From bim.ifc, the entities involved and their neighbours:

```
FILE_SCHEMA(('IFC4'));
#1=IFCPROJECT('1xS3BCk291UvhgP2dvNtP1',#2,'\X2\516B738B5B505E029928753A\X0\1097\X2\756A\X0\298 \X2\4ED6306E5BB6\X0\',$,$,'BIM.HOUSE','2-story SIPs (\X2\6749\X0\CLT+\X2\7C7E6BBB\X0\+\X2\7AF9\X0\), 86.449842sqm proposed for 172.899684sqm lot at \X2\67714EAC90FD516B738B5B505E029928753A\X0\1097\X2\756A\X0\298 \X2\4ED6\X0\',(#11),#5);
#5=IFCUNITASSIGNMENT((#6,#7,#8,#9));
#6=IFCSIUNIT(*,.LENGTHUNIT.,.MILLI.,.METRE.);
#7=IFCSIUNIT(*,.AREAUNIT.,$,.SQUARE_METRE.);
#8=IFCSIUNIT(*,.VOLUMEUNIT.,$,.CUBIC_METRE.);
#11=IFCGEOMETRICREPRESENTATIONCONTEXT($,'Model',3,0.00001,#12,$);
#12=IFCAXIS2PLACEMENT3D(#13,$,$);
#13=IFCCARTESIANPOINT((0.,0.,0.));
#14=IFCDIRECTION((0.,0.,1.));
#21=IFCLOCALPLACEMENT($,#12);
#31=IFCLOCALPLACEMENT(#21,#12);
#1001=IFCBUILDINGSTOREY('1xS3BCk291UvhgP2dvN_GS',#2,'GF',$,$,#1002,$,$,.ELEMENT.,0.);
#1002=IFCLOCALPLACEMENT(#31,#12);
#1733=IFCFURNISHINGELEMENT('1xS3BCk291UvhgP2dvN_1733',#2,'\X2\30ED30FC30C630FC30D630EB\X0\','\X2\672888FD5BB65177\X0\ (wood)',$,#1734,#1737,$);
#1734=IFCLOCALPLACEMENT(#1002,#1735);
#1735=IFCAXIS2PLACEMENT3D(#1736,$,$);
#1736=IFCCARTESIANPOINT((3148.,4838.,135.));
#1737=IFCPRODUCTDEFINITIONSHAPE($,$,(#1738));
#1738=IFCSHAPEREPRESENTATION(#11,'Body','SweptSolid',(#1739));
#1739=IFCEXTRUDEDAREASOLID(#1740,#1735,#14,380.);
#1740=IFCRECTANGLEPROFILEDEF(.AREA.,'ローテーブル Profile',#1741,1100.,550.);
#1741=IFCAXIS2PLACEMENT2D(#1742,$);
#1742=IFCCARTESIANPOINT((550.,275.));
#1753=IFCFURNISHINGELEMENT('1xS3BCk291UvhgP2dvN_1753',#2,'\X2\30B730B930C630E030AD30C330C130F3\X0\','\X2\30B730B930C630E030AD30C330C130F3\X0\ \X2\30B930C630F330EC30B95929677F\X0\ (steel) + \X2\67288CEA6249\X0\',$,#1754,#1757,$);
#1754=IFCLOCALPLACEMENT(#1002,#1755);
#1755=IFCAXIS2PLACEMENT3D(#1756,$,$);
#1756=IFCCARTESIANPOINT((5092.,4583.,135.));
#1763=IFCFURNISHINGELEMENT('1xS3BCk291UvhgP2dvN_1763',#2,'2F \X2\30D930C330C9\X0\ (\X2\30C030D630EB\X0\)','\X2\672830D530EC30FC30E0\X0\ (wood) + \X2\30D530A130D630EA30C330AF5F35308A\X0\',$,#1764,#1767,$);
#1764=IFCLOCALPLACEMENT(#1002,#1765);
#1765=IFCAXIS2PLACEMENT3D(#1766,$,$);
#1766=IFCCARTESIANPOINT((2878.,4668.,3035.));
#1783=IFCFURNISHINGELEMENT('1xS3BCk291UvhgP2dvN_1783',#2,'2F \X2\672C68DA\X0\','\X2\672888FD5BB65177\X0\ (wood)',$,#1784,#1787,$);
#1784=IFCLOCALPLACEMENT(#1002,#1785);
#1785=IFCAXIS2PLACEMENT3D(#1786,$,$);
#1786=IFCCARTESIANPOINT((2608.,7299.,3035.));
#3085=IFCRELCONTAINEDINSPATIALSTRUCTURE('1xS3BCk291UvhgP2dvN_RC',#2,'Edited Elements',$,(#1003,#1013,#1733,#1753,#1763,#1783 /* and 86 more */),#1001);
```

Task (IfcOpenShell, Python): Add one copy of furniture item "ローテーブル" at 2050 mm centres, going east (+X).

```python
import numpy as np
import ifcopenshell
import ifcopenshell.api.geometry
import ifcopenshell.api.root
import ifcopenshell.util.element
import ifcopenshell.util.placement
import ifcopenshell.util.unit

model = ifcopenshell.open("bim.ifc")
unit_scale = ifcopenshell.util.unit.calculate_unit_scale(model)


def reuse_history(source, copy):
    """copy_class also copies each property set's owner history, people and application; keep the originals."""
    for rel in copy.IsDefinedBy:
        if rel.is_a("IfcRelDefinesByProperties") and (history := rel.RelatingPropertyDefinition.OwnerHistory):
            rel.RelatingPropertyDefinition.OwnerHistory = source.OwnerHistory
            ifcopenshell.util.element.remove_deep2(model, history)


source = model.by_guid("1xS3BCk291UvhgP2dvN_1733")
base = ifcopenshell.util.placement.get_local_placement(source.ObjectPlacement)
step = np.array([1.0, 0.0, 0.0]) * 2.05 / unit_scale

for i in range(1, 2):
    copy = ifcopenshell.api.root.copy_class(model, product=source)
    copy.Representation = ifcopenshell.util.element.copy_deep(
        model, source.Representation, exclude=["IfcGeometricRepresentationContext", "IfcRepresentationMap"]
    )
    reuse_history(source, copy)
    matrix = base.copy()
    matrix[:3, 3] += i * step
    print("added at", matrix[:3, 3].round(3) + 0.0)
    ifcopenshell.api.geometry.edit_object_placement(model, product=copy, matrix=matrix, is_si=False)

model.write("bim_v2.ifc")
```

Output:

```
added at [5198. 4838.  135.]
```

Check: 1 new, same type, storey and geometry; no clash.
